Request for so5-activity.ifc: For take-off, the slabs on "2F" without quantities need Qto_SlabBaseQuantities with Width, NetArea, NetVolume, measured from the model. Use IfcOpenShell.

First a look at what the model holds.

```python
import ifcopenshell
import ifcopenshell.util.element
import ifcopenshell.util.unit

model = ifcopenshell.open("so5-activity.ifc")
print(model.schema)
for unit_type in ("LENGTHUNIT", "AREAUNIT", "VOLUMEUNIT"):
    print(unit_type, ifcopenshell.util.unit.calculate_unit_scale(model, unit_type))
storey = next(s for s in model.by_type("IfcBuildingStorey") if s.Name == "2F")
slabs = [e for e in ifcopenshell.util.element.get_decomposition(storey) if e.is_a("IfcSlab")]
for e in sorted(slabs, key=lambda e: e.id()):
    print(e.id(), e.is_a(), e.Name, list(ifcopenshell.util.element.get_psets(e, qtos_only=True)), sep=" | ")
```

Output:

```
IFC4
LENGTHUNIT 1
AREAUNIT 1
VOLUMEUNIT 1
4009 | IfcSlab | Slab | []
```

```python
import ifcopenshell
import ifcopenshell.api.pset
import ifcopenshell.geom
import ifcopenshell.util.element
import ifcopenshell.util.shape
import ifcopenshell.util.unit

model = ifcopenshell.open("so5-activity.ifc")
unit_scale = ifcopenshell.util.unit.calculate_unit_scale(model)
area_scale = ifcopenshell.util.unit.calculate_unit_scale(model, "AREAUNIT")
volume_scale = ifcopenshell.util.unit.calculate_unit_scale(model, "VOLUMEUNIT")
settings = ifcopenshell.geom.settings()

storey = next(s for s in model.by_type("IfcBuildingStorey") if s.Name == "2F")
slabs = [e for e in ifcopenshell.util.element.get_decomposition(storey) if e.is_a("IfcSlab")]

for e in sorted(slabs, key=lambda e: e.id()):
    if ifcopenshell.util.element.get_psets(e, qtos_only=True, should_inherit=False):
        continue
    # Geometry comes back in metres, in the element's own axes.
    shape = ifcopenshell.geom.create_shape(settings, e)
    values = {
        "Width": ifcopenshell.util.shape.get_z(shape.geometry) / unit_scale,
        "NetArea": ifcopenshell.util.shape.get_footprint_area(shape.geometry) / area_scale,
        "NetVolume": ifcopenshell.util.shape.get_volume(shape.geometry) / volume_scale,
    }
    qto = ifcopenshell.api.pset.add_qto(model, product=e, name="Qto_SlabBaseQuantities")
    ifcopenshell.api.pset.edit_qto(model, qto=qto, properties=values)
    print(e.id(), {k: round(v, 3) for k, v in values.items()})

model.write("so5-activity_rev.ifc")
```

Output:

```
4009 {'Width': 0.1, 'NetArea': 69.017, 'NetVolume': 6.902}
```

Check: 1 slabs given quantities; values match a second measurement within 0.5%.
